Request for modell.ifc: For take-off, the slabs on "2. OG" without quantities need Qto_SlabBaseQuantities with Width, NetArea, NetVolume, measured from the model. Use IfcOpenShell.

First a look at what the model holds.

```python
import ifcopenshell
import ifcopenshell.util.element
import ifcopenshell.util.unit

model = ifcopenshell.open("modell.ifc")
print(model.schema)
for unit_type in ("LENGTHUNIT", "AREAUNIT", "VOLUMEUNIT"):
    print(unit_type, ifcopenshell.util.unit.calculate_unit_scale(model, unit_type))
storey = next(s for s in model.by_type("IfcBuildingStorey") if s.Name == "2. OG")
slabs = [e for e in ifcopenshell.util.element.get_decomposition(storey) if e.is_a("IfcSlab")]
for e in sorted(slabs, key=lambda e: e.id()):
    print(e.id(), e.is_a(), e.Name, list(ifcopenshell.util.element.get_psets(e, qtos_only=True)), sep=" | ")
```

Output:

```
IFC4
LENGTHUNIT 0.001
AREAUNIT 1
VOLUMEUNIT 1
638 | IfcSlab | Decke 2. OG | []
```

```python
import ifcopenshell
import ifcopenshell.api.pset
import ifcopenshell.geom
import ifcopenshell.util.element
import ifcopenshell.util.shape
import ifcopenshell.util.unit

model = ifcopenshell.open("modell.ifc")
unit_scale = ifcopenshell.util.unit.calculate_unit_scale(model)
area_scale = ifcopenshell.util.unit.calculate_unit_scale(model, "AREAUNIT")
volume_scale = ifcopenshell.util.unit.calculate_unit_scale(model, "VOLUMEUNIT")
settings = ifcopenshell.geom.settings()

storey = next(s for s in model.by_type("IfcBuildingStorey") if s.Name == "2. OG")
slabs = [e for e in ifcopenshell.util.element.get_decomposition(storey) if e.is_a("IfcSlab")]

for e in sorted(slabs, key=lambda e: e.id()):
    if ifcopenshell.util.element.get_psets(e, qtos_only=True, should_inherit=False):
        continue
    # Geometry comes back in metres, in the element's own axes.
    shape = ifcopenshell.geom.create_shape(settings, e)
    values = {
        "Width": ifcopenshell.util.shape.get_z(shape.geometry) / unit_scale,
        "NetArea": ifcopenshell.util.shape.get_footprint_area(shape.geometry) / area_scale,
        "NetVolume": ifcopenshell.util.shape.get_volume(shape.geometry) / volume_scale,
    }
    qto = ifcopenshell.api.pset.add_qto(model, product=e, name="Qto_SlabBaseQuantities")
    ifcopenshell.api.pset.edit_qto(model, qto=qto, properties=values)
    print(e.id(), {k: round(v, 3) for k, v in values.items()})

model.write("modell_updated.ifc")
```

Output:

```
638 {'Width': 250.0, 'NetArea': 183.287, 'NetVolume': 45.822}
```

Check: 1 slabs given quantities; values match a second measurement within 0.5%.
